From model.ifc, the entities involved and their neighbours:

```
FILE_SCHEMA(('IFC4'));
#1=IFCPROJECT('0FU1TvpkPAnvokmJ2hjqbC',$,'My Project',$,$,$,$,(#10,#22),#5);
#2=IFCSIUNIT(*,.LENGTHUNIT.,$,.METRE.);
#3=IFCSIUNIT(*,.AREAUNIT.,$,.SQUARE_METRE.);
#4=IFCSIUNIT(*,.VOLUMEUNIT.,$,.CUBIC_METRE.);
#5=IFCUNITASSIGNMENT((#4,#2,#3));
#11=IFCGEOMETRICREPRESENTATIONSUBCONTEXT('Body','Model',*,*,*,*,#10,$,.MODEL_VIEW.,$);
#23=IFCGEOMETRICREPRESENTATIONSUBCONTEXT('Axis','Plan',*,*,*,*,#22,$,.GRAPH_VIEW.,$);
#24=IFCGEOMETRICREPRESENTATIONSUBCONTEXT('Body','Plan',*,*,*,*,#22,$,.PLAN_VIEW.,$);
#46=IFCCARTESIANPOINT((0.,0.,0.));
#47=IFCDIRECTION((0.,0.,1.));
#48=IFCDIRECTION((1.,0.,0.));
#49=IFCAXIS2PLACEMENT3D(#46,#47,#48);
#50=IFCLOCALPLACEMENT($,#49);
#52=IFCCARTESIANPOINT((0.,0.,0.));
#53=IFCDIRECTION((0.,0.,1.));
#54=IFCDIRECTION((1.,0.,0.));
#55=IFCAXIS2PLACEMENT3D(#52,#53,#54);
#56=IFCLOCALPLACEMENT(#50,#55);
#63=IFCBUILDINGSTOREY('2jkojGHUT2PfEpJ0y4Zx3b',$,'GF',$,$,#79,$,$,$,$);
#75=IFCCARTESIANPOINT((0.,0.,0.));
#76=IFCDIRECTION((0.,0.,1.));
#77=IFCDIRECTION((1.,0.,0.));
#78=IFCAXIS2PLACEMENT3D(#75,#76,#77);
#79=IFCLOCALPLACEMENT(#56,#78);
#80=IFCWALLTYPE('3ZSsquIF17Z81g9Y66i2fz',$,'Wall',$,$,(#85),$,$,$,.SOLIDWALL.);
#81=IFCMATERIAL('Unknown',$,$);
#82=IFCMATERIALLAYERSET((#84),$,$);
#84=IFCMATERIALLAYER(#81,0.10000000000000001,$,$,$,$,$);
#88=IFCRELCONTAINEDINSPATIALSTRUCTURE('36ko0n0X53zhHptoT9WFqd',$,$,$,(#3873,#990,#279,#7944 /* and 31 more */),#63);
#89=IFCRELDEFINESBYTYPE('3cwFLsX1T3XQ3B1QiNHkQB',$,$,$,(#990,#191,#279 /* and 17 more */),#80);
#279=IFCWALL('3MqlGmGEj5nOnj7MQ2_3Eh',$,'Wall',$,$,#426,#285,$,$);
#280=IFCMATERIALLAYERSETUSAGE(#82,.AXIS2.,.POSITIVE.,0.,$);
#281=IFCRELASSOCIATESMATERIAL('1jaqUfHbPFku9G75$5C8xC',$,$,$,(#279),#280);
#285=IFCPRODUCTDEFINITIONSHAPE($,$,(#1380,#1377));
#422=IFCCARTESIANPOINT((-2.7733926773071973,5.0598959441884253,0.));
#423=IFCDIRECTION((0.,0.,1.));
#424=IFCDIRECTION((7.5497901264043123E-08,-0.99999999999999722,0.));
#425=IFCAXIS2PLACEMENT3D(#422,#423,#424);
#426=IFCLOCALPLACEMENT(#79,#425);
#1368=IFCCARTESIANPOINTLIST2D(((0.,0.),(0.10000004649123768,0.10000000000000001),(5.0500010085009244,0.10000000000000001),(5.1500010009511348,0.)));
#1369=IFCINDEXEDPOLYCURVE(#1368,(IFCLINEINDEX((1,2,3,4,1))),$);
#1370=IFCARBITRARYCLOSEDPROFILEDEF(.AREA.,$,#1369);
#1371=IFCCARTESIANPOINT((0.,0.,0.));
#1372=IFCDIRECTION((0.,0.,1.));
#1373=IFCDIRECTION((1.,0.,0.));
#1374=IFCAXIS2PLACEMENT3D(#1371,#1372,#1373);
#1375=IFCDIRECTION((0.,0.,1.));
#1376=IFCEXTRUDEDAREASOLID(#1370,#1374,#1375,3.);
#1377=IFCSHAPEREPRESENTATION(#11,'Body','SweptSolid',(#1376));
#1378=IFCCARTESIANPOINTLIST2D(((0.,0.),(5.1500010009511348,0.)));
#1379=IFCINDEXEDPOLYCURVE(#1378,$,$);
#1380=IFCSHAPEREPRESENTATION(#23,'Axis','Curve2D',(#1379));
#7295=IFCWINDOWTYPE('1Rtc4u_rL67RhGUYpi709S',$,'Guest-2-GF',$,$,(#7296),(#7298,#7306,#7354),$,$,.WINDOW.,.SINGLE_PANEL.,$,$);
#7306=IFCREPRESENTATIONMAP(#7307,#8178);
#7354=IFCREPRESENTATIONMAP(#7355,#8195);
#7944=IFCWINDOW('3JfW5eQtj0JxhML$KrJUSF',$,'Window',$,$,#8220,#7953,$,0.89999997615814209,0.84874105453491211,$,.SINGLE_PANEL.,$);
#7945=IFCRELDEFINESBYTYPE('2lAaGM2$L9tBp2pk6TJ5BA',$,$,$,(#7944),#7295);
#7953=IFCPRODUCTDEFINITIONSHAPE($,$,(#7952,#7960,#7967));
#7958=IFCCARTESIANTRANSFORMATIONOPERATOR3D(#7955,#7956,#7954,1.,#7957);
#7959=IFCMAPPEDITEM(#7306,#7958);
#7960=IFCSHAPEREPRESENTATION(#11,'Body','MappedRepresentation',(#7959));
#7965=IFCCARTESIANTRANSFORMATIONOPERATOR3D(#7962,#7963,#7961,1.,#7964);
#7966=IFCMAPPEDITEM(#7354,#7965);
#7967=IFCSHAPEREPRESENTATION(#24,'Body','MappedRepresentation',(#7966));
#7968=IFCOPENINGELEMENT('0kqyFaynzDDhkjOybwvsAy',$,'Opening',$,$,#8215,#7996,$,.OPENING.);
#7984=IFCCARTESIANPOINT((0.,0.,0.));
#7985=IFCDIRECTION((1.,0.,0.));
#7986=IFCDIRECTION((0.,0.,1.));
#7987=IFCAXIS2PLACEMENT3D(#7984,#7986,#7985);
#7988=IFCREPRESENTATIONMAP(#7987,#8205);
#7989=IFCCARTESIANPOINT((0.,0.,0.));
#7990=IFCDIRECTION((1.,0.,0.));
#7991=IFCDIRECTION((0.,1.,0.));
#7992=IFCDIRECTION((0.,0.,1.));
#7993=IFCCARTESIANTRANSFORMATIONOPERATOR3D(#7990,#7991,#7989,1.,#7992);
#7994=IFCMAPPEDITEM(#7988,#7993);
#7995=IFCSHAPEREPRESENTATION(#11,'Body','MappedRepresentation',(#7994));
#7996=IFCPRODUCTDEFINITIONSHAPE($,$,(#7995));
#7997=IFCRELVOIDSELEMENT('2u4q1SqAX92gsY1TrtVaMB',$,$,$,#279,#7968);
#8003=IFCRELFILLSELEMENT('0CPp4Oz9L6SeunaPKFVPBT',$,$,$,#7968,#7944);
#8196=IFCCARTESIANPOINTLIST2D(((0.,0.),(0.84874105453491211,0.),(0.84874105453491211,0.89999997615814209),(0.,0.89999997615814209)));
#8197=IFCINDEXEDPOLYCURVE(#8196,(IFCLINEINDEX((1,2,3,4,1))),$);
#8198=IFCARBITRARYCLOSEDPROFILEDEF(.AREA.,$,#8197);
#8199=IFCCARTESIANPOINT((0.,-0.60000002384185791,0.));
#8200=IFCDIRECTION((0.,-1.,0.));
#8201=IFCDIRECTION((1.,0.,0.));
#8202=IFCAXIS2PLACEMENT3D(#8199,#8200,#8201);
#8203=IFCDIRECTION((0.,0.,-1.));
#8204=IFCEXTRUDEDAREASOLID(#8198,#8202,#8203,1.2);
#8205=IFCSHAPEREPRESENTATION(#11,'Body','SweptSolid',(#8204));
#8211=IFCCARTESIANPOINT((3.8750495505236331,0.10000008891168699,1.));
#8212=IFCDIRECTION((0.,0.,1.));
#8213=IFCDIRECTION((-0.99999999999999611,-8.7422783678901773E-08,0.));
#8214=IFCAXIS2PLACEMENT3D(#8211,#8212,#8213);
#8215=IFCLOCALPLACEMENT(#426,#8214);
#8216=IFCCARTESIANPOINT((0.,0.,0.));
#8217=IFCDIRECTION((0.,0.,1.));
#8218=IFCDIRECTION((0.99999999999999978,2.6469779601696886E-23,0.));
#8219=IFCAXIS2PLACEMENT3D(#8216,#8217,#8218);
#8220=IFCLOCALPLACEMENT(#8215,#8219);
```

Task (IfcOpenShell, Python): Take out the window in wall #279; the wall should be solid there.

```python
import ifcopenshell
import ifcopenshell.api.feature
import ifcopenshell.api.root
import ifcopenshell.geom
import ifcopenshell.util.shape

model = ifcopenshell.open("model.ifc")
settings = ifcopenshell.geom.settings()


def volume(element):
    """Net volume in cubic metres, openings subtracted."""
    shape = ifcopenshell.geom.create_shape(settings, element)
    return ifcopenshell.util.shape.get_volume(shape.geometry)


window = model.by_guid("3JfW5eQtj0JxhML$KrJUSF")
opening = window.FillsVoids[0].RelatingOpeningElement
wall = opening.VoidsElements[0].RelatingBuildingElement
before = volume(wall)

ifcopenshell.api.root.remove_product(model, product=window)
ifcopenshell.api.feature.remove_feature(model, feature=opening)

after = volume(wall)

print(f"wall volume {before:.3f} -> {after:.3f} m3")

model.write("model_updated.ifc")
```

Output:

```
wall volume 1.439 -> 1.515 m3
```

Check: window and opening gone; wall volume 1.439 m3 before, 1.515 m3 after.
